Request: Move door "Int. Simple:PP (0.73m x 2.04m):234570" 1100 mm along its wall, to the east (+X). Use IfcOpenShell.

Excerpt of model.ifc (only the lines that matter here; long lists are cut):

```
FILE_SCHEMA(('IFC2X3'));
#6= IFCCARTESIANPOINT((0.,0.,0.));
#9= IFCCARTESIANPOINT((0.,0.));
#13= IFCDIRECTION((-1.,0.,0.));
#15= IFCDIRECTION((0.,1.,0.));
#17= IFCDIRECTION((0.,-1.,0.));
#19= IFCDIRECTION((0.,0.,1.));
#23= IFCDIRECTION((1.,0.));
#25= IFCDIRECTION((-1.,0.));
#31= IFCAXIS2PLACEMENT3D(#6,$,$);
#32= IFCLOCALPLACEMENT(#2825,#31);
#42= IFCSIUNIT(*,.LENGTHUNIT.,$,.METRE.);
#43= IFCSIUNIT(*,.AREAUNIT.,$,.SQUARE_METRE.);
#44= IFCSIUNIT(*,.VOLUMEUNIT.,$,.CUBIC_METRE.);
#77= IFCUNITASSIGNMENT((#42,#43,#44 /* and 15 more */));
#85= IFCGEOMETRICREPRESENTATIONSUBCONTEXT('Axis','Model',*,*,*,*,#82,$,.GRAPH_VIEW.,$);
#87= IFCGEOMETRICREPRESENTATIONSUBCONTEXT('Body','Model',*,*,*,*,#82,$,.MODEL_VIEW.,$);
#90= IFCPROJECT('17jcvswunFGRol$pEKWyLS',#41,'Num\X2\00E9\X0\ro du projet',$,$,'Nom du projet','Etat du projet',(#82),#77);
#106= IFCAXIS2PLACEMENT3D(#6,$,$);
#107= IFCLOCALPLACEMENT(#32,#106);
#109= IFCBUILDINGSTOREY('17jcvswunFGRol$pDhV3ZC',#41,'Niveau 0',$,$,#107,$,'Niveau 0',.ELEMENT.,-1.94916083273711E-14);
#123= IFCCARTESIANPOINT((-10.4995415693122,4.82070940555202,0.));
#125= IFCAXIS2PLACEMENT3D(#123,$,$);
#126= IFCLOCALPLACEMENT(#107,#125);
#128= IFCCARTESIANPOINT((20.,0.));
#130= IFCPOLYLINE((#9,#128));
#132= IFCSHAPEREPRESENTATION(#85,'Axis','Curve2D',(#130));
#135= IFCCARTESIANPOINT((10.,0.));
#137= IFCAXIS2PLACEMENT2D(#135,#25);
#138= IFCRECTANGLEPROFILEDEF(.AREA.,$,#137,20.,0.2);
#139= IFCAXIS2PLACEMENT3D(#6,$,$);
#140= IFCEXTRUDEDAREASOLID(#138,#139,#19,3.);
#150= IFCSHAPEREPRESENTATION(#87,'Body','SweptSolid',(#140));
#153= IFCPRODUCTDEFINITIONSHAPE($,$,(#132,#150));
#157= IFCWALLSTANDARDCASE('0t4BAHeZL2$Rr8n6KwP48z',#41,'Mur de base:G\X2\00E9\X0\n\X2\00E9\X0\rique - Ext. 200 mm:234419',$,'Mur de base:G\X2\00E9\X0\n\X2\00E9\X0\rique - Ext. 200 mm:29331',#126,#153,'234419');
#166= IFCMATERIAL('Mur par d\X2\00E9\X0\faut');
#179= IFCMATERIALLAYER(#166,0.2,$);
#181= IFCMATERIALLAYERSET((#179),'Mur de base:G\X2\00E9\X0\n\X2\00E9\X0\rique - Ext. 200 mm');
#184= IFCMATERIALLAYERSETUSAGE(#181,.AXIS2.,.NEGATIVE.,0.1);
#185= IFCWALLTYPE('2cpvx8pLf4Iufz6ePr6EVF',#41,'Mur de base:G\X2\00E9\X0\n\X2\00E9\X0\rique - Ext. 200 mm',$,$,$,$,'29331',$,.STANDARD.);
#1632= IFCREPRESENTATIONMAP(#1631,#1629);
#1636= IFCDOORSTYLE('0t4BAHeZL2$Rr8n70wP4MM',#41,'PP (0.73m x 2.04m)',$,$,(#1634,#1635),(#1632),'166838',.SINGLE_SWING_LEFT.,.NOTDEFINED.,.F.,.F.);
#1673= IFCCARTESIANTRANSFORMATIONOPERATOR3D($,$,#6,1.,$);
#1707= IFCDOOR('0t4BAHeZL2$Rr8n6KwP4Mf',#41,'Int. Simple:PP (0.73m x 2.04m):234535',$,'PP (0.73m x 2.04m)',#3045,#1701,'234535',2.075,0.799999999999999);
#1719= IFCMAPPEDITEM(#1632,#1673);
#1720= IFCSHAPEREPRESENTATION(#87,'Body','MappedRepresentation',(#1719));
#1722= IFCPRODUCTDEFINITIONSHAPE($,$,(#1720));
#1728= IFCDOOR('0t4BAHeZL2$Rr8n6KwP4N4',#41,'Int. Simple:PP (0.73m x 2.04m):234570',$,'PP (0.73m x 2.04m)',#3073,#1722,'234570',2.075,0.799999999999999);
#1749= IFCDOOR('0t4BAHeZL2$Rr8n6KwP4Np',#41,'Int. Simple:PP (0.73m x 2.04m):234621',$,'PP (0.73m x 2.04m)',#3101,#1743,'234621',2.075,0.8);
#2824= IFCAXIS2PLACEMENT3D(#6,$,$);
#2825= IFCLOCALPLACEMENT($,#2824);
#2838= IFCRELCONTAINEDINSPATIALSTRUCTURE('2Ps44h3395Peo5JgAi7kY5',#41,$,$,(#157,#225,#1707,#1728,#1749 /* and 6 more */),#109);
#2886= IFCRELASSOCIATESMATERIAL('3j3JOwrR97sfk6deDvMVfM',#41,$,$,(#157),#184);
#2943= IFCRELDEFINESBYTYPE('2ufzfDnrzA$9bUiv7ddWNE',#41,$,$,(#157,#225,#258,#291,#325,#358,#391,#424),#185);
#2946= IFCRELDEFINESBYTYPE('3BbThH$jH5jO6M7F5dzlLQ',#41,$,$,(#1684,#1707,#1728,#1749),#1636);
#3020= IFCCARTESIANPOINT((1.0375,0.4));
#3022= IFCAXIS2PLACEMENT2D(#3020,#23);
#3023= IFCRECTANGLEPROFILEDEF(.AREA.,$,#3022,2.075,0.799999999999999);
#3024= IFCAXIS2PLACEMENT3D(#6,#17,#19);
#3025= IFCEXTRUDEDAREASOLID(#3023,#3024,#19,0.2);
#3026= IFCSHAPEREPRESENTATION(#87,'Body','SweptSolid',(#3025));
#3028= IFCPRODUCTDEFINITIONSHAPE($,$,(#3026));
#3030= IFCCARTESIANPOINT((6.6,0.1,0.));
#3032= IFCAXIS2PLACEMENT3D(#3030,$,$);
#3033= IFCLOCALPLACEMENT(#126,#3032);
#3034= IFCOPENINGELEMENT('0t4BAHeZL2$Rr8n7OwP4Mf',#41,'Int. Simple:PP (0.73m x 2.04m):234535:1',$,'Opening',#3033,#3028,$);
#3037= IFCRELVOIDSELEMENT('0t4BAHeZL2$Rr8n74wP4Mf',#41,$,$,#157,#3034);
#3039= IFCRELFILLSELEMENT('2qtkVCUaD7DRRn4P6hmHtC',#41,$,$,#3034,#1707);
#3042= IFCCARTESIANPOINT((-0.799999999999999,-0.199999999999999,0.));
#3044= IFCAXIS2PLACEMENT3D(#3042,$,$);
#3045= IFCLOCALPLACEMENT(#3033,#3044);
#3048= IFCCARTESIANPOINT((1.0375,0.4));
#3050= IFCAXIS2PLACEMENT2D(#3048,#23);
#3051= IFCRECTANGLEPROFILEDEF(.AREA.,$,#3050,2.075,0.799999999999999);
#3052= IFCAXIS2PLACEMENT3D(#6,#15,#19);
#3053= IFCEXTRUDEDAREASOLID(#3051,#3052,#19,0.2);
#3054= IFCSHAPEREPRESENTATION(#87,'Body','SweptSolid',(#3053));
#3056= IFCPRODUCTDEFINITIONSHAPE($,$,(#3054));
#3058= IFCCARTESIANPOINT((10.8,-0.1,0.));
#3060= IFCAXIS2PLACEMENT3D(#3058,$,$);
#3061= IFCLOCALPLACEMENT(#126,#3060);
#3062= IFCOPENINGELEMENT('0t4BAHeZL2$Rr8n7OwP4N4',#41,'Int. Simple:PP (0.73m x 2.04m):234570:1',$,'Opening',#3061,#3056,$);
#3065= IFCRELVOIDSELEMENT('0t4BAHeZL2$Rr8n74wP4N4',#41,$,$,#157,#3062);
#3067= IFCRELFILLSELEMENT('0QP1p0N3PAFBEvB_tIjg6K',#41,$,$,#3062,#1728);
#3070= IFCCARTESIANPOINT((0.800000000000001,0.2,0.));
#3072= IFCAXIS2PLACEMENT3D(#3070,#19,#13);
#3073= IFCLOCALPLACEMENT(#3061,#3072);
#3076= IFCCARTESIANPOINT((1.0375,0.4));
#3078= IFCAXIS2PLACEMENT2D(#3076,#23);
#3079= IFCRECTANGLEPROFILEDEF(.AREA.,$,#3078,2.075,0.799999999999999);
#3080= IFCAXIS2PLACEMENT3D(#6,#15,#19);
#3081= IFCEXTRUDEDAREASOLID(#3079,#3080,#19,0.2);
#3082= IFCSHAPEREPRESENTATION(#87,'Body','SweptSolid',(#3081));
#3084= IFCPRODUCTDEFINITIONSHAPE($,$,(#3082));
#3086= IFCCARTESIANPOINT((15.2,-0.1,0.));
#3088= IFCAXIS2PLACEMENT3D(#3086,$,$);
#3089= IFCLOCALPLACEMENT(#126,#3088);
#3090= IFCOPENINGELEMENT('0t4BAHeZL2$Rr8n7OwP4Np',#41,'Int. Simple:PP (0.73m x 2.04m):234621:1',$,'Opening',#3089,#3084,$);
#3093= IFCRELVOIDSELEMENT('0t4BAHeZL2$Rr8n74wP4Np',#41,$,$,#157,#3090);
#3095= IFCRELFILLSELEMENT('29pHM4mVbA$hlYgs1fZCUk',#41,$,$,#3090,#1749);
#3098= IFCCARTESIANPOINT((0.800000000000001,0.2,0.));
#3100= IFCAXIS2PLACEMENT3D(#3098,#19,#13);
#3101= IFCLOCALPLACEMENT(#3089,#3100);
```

```python
import ifcopenshell
import ifcopenshell.api.geometry
import ifcopenshell.util.placement
import ifcopenshell.util.unit

model = ifcopenshell.open("model.ifc")
unit_scale = ifcopenshell.util.unit.calculate_unit_scale(model)

door = model.by_guid("0t4BAHeZL2$Rr8n6KwP4N4")
opening = door.FillsVoids[0].RelatingOpeningElement
wall = opening.VoidsElements[0].RelatingBuildingElement

wall_matrix = ifcopenshell.util.placement.get_local_placement(wall.ObjectPlacement)
shift = wall_matrix[:3, 0] * 1.1 / unit_scale
before = ifcopenshell.util.placement.get_local_placement(door.ObjectPlacement)[:3, 3].copy()

# The door is placed relative to its opening, so it follows when the opening moves.
matrix = ifcopenshell.util.placement.get_local_placement(opening.ObjectPlacement)
matrix[:3, 3] += shift
ifcopenshell.api.geometry.edit_object_placement(
    model, product=opening, matrix=matrix, is_si=False, should_transform_children=True
)

after = ifcopenshell.util.placement.get_local_placement(door.ObjectPlacement)[:3, 3]
print("door moved by", (after - before).round(3) + 0.0)

model.write("model-out.ifc")
```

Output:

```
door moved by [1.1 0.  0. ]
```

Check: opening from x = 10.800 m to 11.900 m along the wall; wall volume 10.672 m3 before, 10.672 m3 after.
